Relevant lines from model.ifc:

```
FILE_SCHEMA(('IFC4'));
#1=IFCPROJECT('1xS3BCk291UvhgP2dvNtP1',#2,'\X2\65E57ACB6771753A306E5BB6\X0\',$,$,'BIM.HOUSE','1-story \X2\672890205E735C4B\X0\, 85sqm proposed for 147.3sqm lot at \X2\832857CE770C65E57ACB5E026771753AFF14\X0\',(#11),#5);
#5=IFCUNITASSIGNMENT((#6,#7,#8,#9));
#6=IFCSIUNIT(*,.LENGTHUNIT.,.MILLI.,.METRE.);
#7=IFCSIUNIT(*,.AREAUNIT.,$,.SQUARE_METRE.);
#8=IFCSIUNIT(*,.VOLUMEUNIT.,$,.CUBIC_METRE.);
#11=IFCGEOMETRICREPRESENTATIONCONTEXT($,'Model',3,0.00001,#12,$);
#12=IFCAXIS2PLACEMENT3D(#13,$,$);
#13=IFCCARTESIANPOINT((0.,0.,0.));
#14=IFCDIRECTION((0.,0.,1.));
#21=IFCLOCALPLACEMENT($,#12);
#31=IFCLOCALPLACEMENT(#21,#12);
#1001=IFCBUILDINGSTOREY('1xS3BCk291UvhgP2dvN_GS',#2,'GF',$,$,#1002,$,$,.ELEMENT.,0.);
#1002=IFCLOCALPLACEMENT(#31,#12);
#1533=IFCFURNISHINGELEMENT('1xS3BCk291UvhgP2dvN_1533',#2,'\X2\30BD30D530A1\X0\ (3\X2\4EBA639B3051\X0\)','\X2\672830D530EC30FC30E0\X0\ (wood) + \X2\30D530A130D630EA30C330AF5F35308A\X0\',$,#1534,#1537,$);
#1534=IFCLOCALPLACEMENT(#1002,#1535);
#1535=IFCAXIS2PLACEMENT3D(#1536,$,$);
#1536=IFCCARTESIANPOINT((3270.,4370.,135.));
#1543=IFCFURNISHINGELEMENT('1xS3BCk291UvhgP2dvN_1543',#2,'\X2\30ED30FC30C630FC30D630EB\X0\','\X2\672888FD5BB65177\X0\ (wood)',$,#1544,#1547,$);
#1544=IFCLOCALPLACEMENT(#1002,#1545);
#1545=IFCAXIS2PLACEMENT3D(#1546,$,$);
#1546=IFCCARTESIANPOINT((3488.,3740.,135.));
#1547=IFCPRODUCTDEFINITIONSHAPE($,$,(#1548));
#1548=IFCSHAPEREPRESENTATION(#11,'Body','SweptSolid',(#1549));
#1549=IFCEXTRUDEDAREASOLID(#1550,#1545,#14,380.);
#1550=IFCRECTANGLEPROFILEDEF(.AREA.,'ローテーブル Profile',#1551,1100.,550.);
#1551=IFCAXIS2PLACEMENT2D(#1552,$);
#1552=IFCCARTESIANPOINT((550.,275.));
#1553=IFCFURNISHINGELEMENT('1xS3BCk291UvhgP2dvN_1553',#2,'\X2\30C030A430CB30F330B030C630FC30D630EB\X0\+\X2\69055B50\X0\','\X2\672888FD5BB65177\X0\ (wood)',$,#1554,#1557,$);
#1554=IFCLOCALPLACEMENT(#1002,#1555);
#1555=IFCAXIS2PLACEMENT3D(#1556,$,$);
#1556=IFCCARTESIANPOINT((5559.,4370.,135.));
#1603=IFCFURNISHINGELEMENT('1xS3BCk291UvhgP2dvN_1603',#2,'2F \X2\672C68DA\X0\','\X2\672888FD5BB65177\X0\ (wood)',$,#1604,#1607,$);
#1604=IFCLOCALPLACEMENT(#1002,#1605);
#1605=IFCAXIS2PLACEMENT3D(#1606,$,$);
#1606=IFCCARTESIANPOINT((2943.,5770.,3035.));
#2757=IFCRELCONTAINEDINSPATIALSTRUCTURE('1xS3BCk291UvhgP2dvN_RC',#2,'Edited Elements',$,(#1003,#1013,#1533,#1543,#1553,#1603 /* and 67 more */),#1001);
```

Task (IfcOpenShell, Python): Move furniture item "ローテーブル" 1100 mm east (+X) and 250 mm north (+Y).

```python
import ifcopenshell
import ifcopenshell.api.geometry
import ifcopenshell.util.placement
import ifcopenshell.util.unit

model = ifcopenshell.open("model.ifc")
unit_scale = ifcopenshell.util.unit.calculate_unit_scale(model)

item = model.by_guid("1xS3BCk291UvhgP2dvN_1543")
matrix = ifcopenshell.util.placement.get_local_placement(item.ObjectPlacement)
matrix[0, 3] += 1.1 / unit_scale
matrix[1, 3] += 0.25 / unit_scale
ifcopenshell.api.geometry.edit_object_placement(model, product=item, matrix=matrix, is_si=False)

print(ifcopenshell.util.placement.get_local_placement(item.ObjectPlacement).round(3) + 0.0)

model.write("model_edited.ifc")
```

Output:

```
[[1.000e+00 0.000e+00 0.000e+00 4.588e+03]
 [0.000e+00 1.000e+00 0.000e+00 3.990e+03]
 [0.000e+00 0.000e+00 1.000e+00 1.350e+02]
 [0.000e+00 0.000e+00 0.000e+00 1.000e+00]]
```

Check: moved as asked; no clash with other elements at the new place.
